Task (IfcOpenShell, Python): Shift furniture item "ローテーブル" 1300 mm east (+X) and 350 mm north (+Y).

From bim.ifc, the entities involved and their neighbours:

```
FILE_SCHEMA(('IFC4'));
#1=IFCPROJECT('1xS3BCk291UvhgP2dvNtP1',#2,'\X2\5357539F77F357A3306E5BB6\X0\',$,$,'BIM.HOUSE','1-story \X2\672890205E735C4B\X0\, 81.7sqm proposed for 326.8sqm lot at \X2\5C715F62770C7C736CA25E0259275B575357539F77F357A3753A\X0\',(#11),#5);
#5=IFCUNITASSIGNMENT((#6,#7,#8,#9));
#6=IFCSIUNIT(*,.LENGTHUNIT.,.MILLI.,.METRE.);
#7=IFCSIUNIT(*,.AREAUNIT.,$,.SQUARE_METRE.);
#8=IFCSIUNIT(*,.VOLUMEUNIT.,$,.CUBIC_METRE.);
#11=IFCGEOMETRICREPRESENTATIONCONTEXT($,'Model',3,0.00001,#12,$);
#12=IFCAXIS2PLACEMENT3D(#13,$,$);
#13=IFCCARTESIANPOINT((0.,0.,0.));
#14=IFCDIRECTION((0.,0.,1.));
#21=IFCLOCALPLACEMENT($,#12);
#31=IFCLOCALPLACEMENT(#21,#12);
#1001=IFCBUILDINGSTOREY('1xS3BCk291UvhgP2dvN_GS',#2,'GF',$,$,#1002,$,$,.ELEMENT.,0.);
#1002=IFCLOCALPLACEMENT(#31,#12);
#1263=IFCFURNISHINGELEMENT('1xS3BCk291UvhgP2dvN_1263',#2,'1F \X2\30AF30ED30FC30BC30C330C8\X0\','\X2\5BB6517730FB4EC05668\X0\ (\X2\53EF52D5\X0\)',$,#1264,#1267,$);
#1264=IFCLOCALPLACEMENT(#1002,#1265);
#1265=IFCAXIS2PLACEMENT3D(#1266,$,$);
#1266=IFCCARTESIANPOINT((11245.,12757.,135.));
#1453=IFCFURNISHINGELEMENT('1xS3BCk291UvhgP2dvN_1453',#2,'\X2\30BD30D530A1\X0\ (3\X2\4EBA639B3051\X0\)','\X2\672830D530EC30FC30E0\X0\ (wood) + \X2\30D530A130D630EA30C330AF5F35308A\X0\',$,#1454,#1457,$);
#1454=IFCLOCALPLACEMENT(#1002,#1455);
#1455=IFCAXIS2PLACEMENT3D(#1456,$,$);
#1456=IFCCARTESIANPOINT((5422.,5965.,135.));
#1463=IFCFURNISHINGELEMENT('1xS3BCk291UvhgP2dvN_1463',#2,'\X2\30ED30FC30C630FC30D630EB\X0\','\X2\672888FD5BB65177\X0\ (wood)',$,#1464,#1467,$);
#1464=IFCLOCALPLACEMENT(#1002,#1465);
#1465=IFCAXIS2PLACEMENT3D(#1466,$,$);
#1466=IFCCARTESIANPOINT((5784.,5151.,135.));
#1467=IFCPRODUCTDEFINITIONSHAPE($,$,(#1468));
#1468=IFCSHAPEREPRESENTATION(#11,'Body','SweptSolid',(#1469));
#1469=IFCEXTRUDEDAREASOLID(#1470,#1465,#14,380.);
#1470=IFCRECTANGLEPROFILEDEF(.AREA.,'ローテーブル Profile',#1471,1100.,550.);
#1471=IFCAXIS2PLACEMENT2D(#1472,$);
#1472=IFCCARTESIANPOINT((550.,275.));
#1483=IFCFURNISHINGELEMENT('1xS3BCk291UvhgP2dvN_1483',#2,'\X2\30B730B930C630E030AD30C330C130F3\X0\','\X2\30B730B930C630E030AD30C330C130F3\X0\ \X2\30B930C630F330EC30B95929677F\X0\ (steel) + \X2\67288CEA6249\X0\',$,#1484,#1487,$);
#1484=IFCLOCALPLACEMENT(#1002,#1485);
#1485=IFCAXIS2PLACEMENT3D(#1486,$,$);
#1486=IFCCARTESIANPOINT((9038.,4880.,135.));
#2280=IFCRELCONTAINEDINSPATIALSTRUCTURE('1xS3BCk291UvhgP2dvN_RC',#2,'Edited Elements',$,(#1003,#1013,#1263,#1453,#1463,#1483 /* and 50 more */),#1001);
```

```python
import ifcopenshell
import ifcopenshell.api.geometry
import ifcopenshell.util.placement

model = ifcopenshell.open("bim.ifc")

item = model.by_guid("1xS3BCk291UvhgP2dvN_1463")
matrix = ifcopenshell.util.placement.get_local_placement(item.ObjectPlacement)
matrix[0, 3] += 1300.0
matrix[1, 3] += 350.0
ifcopenshell.api.geometry.edit_object_placement(model, product=item, matrix=matrix, is_si=False)

print(ifcopenshell.util.placement.get_local_placement(item.ObjectPlacement).round(3) + 0.0)

model.write("bim_edited.ifc")
```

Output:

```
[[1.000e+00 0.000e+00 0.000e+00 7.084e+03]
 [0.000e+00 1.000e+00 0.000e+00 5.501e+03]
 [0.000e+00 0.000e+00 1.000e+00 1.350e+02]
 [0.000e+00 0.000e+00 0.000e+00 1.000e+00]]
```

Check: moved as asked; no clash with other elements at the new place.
